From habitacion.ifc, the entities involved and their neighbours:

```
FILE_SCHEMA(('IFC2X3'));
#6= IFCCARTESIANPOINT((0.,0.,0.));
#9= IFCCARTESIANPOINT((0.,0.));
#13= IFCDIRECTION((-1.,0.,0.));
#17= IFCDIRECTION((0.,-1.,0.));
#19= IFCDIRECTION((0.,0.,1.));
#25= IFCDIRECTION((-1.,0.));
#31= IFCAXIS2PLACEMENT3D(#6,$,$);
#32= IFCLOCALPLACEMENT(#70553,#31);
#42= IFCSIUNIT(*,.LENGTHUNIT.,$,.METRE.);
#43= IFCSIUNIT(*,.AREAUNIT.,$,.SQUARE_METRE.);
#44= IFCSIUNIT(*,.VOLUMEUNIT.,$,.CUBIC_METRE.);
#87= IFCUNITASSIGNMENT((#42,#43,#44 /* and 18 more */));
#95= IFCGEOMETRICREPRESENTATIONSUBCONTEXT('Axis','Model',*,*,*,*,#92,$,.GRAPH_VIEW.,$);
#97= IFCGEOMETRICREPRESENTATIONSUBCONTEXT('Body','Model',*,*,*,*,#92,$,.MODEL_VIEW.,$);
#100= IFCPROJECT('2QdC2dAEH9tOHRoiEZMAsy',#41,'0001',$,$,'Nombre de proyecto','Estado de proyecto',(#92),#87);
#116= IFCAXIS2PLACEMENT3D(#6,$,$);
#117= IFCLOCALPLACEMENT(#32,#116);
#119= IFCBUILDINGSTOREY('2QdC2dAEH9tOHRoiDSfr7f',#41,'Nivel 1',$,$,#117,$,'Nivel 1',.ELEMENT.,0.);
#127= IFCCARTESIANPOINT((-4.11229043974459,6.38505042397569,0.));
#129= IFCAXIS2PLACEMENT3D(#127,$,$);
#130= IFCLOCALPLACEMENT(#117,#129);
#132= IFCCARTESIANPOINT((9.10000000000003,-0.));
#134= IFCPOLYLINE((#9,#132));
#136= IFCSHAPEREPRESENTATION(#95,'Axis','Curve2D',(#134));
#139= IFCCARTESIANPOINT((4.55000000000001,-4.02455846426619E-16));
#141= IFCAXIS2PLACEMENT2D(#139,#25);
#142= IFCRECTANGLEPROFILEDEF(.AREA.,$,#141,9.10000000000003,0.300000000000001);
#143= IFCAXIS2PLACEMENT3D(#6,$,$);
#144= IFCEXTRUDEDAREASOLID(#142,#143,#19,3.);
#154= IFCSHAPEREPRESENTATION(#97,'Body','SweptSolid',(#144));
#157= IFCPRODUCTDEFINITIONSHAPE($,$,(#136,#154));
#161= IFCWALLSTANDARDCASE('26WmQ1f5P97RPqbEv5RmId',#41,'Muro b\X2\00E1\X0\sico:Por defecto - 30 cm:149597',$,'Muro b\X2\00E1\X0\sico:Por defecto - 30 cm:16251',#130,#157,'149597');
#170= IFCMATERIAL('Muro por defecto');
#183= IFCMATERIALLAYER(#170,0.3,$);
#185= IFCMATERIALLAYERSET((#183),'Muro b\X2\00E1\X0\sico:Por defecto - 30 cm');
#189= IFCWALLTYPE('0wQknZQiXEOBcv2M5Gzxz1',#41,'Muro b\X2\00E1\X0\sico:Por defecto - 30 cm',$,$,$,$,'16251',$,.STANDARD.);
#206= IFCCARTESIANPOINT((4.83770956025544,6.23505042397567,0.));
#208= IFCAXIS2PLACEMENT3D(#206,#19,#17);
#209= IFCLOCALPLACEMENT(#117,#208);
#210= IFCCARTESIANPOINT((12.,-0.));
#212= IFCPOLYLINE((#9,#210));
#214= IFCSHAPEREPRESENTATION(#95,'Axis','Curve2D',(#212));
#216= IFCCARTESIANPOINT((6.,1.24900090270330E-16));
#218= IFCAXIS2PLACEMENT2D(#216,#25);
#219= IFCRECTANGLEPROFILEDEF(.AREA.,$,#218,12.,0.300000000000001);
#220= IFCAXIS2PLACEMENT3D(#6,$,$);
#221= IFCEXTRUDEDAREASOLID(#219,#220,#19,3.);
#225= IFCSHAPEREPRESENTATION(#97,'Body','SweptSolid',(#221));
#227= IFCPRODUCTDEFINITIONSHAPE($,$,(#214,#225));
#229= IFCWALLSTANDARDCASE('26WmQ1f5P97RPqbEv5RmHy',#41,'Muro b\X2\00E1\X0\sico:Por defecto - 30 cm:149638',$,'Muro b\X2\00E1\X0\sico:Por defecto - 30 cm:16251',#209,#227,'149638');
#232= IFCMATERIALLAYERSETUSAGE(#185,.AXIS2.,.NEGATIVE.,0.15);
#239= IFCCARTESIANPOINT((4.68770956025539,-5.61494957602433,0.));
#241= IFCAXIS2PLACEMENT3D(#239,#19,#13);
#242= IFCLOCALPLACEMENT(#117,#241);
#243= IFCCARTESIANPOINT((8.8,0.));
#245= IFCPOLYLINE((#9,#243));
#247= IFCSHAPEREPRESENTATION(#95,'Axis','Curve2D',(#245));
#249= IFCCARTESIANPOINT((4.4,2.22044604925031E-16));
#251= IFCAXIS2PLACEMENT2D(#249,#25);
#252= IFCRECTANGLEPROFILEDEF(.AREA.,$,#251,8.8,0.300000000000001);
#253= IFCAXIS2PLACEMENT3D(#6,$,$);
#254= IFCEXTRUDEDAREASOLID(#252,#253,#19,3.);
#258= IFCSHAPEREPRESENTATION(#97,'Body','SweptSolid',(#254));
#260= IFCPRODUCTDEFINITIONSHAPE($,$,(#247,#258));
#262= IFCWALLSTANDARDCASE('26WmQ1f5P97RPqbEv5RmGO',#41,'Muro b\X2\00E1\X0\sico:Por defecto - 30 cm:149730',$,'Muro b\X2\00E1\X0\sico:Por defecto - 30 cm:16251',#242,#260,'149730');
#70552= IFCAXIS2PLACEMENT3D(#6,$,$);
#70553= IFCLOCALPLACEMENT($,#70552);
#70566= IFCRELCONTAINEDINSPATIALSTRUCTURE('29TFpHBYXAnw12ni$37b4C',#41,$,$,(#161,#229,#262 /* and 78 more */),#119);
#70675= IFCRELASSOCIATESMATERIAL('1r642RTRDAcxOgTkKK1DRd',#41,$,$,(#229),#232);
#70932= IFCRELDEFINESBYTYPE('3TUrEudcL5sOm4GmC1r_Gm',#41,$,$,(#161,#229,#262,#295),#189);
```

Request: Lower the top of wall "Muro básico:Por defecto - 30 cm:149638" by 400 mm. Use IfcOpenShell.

```python
import ifcopenshell
import ifcopenshell.geom
import ifcopenshell.util.representation
import ifcopenshell.util.shape

model = ifcopenshell.open("habitacion.ifc")
settings = ifcopenshell.geom.settings()


def volume(element):
    """Net volume in cubic metres, openings subtracted."""
    shape = ifcopenshell.geom.create_shape(settings, element)
    return ifcopenshell.util.shape.get_volume(shape.geometry)


wall = model.by_guid("26WmQ1f5P97RPqbEv5RmHy")
before = volume(wall)

body = ifcopenshell.util.representation.get_representation(wall, "Model", "Body")
solid = body.Items[0]
old_height = solid.Depth
solid.Depth -= 0.4
after = volume(wall)

print(f"height {old_height:g} -> {solid.Depth:g}, volume {before:.3f} -> {after:.3f} m3")

model.write("habitacion_rev.ifc")
```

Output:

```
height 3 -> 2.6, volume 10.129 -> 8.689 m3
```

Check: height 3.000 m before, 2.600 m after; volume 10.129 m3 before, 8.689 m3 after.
